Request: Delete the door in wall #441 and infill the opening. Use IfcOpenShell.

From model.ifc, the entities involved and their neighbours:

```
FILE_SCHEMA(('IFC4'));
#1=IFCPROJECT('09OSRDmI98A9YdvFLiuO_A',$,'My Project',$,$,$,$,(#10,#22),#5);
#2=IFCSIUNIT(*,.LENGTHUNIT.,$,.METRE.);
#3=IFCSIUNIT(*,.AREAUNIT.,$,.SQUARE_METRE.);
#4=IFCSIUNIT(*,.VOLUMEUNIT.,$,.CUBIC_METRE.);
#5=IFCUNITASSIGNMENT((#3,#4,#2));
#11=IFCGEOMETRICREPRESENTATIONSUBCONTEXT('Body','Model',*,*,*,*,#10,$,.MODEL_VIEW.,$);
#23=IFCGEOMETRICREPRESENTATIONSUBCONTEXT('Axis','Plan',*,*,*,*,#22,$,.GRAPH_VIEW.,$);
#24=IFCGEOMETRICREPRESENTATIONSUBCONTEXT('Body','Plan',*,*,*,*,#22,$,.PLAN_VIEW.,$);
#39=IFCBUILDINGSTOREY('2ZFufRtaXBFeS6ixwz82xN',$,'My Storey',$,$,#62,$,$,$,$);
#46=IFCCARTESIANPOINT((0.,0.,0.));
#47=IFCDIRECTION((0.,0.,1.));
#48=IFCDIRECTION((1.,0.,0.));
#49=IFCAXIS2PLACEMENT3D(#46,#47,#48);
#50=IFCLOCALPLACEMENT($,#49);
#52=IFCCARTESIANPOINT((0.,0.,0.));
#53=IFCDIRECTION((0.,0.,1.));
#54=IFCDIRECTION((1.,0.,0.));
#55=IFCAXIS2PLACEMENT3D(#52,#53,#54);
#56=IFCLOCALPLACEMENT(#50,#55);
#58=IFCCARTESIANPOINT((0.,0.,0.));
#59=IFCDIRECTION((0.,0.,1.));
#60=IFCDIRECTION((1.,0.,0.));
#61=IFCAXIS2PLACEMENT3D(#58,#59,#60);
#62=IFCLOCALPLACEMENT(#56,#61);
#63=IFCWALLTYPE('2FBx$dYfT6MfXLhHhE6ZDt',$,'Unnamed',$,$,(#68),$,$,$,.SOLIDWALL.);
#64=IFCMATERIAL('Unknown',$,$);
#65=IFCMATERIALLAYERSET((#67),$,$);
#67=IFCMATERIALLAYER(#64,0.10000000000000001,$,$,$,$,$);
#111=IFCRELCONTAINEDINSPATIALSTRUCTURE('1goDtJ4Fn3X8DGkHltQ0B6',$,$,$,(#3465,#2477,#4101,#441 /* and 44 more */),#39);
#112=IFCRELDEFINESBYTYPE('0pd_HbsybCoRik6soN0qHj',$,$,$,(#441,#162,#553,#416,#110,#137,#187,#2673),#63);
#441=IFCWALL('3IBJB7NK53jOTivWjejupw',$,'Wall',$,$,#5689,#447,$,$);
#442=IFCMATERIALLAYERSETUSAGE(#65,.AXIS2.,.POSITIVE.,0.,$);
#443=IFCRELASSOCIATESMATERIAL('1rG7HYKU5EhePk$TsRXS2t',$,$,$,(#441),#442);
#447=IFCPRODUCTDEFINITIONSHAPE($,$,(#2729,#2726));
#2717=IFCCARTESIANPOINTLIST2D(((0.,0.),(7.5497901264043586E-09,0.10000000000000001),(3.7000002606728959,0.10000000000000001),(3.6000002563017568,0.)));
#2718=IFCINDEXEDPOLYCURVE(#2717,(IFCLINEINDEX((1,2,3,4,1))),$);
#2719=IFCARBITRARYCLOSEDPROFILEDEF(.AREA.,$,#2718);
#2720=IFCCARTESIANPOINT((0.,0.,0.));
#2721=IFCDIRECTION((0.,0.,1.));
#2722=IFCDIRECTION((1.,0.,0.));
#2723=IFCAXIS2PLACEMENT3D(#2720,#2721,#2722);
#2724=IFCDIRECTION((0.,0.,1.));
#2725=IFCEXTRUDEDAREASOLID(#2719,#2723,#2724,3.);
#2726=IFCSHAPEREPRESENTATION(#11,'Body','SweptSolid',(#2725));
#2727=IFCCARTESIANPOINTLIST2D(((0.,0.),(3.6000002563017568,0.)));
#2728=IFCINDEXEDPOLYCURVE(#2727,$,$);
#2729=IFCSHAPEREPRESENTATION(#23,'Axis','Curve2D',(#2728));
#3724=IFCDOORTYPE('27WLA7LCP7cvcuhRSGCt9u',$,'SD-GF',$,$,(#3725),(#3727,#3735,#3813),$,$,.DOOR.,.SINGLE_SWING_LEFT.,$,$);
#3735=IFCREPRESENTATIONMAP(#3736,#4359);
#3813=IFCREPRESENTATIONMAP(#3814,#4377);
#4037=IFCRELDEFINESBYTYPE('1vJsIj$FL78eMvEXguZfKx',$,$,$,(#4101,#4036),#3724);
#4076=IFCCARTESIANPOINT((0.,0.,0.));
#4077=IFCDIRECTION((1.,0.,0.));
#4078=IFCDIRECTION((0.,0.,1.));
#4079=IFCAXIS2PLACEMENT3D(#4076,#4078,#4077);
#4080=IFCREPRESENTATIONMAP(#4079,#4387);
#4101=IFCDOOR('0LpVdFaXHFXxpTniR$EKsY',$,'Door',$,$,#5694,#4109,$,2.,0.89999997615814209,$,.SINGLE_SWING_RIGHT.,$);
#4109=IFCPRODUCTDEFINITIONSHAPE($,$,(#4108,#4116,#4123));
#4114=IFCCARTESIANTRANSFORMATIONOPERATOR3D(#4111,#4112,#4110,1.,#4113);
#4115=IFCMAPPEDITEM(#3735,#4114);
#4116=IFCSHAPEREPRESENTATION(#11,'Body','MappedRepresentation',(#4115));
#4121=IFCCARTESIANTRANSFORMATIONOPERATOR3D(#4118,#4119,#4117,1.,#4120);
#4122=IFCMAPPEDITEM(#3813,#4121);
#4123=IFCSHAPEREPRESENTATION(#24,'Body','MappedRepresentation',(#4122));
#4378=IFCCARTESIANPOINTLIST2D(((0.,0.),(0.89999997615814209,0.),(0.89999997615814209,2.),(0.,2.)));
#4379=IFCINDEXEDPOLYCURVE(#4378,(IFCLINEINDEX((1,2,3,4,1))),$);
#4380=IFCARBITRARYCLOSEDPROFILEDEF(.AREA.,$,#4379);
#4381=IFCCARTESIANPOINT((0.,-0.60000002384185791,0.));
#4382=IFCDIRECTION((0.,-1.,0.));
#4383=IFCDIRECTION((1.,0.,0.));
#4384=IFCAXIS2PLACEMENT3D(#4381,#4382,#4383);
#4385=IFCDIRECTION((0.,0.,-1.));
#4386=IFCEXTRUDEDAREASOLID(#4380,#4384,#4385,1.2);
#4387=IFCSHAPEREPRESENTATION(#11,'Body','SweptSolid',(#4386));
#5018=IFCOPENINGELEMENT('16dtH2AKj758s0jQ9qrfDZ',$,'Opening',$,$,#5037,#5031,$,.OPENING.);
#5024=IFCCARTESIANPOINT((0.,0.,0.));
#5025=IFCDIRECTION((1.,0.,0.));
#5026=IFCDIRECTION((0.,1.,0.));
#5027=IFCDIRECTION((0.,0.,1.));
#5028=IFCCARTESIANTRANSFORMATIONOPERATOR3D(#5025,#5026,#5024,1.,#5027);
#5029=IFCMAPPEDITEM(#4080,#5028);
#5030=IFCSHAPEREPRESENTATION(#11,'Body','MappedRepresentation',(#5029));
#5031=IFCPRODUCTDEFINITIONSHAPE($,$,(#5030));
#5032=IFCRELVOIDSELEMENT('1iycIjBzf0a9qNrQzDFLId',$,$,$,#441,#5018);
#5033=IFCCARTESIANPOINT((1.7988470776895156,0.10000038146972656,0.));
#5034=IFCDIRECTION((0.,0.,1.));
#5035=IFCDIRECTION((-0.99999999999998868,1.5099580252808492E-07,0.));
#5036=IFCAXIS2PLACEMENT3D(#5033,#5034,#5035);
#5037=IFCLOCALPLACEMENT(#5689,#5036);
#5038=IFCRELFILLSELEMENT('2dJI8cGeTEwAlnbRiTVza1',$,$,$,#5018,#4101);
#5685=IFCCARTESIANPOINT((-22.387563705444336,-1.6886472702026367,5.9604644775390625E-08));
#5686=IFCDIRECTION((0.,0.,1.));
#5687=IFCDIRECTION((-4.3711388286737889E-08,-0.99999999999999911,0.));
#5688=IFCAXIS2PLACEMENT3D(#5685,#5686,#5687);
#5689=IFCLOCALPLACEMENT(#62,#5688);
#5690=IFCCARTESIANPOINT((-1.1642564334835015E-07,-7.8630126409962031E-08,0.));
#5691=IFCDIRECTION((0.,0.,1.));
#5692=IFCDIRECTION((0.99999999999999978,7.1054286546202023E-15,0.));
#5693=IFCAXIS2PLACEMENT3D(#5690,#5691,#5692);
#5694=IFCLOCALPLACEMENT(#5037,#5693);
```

```python
import ifcopenshell
import ifcopenshell.api.feature
import ifcopenshell.api.root
import ifcopenshell.geom
import ifcopenshell.util.shape

model = ifcopenshell.open("model.ifc")
settings = ifcopenshell.geom.settings()


def volume(element):
    """Net volume in cubic metres, openings subtracted."""
    shape = ifcopenshell.geom.create_shape(settings, element)
    return ifcopenshell.util.shape.get_volume(shape.geometry)


door = model.by_id(4101)
opening = door.FillsVoids[0].RelatingOpeningElement
wall = opening.VoidsElements[0].RelatingBuildingElement
before = volume(wall)

ifcopenshell.api.root.remove_product(model, product=door)
ifcopenshell.api.feature.remove_feature(model, feature=opening)

after = volume(wall)

print(f"wall volume {before:.3f} -> {after:.3f} m3")

model.write("model_edited.ifc")
```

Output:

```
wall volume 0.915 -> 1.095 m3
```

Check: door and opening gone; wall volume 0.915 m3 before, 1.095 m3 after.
